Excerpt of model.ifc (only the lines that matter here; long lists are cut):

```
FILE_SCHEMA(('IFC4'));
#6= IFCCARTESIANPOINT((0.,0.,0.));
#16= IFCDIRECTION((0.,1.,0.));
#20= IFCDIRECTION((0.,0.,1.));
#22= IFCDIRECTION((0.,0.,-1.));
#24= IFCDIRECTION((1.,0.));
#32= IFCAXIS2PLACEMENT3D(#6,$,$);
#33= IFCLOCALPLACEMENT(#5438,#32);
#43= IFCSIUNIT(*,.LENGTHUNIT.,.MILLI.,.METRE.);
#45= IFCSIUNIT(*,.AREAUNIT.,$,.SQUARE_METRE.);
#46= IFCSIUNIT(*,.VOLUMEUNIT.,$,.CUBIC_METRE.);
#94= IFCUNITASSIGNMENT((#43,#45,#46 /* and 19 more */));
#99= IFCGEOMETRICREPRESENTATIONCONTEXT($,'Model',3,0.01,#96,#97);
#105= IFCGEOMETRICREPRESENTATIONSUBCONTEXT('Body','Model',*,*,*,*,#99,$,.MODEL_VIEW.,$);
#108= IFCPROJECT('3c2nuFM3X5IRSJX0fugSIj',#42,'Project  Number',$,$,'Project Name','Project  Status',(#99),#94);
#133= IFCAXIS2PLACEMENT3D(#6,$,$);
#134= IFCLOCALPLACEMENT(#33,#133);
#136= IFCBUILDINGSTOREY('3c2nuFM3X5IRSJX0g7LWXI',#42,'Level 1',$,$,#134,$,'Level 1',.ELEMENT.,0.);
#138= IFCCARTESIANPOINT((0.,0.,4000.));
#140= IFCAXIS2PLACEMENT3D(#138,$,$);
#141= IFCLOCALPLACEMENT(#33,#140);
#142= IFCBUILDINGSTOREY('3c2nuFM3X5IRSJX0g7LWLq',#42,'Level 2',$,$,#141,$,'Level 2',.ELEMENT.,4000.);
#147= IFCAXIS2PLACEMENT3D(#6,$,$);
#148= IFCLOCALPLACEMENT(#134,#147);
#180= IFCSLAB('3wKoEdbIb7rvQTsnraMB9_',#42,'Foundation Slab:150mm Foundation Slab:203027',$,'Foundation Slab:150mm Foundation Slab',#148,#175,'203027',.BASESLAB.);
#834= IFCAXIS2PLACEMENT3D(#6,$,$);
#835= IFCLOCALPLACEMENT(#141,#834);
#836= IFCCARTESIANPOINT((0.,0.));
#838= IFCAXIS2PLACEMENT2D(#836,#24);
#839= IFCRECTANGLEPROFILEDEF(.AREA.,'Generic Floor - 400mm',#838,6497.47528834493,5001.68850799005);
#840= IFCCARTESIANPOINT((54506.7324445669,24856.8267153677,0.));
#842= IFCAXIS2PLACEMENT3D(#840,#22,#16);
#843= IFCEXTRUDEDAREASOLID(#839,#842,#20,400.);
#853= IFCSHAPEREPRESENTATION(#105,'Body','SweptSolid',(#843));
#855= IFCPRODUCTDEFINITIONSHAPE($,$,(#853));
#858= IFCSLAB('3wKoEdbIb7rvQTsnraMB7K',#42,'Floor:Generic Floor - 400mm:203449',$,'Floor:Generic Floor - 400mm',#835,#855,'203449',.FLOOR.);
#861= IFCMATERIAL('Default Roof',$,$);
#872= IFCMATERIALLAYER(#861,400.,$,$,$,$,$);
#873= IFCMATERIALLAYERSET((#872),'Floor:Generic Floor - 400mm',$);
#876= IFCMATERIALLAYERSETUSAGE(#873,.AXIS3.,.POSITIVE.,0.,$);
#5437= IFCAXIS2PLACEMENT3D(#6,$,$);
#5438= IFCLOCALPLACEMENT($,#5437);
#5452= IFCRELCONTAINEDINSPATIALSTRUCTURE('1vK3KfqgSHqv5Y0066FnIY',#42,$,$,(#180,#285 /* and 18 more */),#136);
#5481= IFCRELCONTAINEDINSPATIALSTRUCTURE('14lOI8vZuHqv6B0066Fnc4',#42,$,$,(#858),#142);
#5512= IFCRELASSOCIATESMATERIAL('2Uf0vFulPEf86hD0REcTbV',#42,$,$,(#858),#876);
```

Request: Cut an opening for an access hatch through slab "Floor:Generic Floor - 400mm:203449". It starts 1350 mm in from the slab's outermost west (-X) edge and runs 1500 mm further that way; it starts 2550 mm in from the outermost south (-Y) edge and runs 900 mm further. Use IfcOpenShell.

```python
import numpy as np
import ifcopenshell
import ifcopenshell.api.feature
import ifcopenshell.api.geometry
import ifcopenshell.api.root
import ifcopenshell.geom
import ifcopenshell.util.placement
import ifcopenshell.util.representation
import ifcopenshell.util.shape
import ifcopenshell.util.unit

model = ifcopenshell.open("model.ifc")
unit_scale = ifcopenshell.util.unit.calculate_unit_scale(model)
settings = ifcopenshell.geom.settings()


def volume(element):
    """Net volume in cubic metres, openings subtracted."""
    shape = ifcopenshell.geom.create_shape(settings, element)
    return ifcopenshell.util.shape.get_volume(shape.geometry)


slab = model.by_guid("3wKoEdbIb7rvQTsnraMB7K")
before = volume(slab)

# Extent in the slab's own axes, in metres. The edges named are its -X and -Y sides.
slab_shape = ifcopenshell.geom.create_shape(settings, slab)
vertices = ifcopenshell.util.shape.get_vertices(slab_shape.geometry)
x_min, y_min, bottom = vertices.min(axis=0)
top = vertices[:, 2].max()

opening = ifcopenshell.api.root.create_entity(model, ifc_class="IfcOpeningElement", name="Access hatch opening", predefined_type="OPENING")
context = ifcopenshell.util.representation.get_context(model, "Model", "Body", "MODEL_VIEW")
width, depth = 1.5, 0.9
outline = [(0.0, 0.0), (width, 0.0), (width, depth), (0.0, depth), (0.0, 0.0)]
# Overshoot both faces by 50 mm so the cut is clean.
shape = ifcopenshell.api.geometry.add_slab_representation(
    model, context=context, depth=top - bottom + 0.1, polyline=outline
)
ifcopenshell.api.geometry.assign_representation(model, product=opening, representation=shape)

matrix = ifcopenshell.util.placement.get_local_placement(slab.ObjectPlacement)
matrix[:, 3] = matrix @ np.append(np.array([x_min + 1.35, y_min + 2.55, bottom - 0.05]) / unit_scale, 1.0)
ifcopenshell.api.geometry.edit_object_placement(model, product=opening, matrix=matrix, is_si=False)
ifcopenshell.api.feature.add_feature(model, feature=opening, element=slab)

after = volume(slab)

print(f"slab volume {before:.3f} -> {after:.3f} m3")

model.write("model_v2.ifc")
```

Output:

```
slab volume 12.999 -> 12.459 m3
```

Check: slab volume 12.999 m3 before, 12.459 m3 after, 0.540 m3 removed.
